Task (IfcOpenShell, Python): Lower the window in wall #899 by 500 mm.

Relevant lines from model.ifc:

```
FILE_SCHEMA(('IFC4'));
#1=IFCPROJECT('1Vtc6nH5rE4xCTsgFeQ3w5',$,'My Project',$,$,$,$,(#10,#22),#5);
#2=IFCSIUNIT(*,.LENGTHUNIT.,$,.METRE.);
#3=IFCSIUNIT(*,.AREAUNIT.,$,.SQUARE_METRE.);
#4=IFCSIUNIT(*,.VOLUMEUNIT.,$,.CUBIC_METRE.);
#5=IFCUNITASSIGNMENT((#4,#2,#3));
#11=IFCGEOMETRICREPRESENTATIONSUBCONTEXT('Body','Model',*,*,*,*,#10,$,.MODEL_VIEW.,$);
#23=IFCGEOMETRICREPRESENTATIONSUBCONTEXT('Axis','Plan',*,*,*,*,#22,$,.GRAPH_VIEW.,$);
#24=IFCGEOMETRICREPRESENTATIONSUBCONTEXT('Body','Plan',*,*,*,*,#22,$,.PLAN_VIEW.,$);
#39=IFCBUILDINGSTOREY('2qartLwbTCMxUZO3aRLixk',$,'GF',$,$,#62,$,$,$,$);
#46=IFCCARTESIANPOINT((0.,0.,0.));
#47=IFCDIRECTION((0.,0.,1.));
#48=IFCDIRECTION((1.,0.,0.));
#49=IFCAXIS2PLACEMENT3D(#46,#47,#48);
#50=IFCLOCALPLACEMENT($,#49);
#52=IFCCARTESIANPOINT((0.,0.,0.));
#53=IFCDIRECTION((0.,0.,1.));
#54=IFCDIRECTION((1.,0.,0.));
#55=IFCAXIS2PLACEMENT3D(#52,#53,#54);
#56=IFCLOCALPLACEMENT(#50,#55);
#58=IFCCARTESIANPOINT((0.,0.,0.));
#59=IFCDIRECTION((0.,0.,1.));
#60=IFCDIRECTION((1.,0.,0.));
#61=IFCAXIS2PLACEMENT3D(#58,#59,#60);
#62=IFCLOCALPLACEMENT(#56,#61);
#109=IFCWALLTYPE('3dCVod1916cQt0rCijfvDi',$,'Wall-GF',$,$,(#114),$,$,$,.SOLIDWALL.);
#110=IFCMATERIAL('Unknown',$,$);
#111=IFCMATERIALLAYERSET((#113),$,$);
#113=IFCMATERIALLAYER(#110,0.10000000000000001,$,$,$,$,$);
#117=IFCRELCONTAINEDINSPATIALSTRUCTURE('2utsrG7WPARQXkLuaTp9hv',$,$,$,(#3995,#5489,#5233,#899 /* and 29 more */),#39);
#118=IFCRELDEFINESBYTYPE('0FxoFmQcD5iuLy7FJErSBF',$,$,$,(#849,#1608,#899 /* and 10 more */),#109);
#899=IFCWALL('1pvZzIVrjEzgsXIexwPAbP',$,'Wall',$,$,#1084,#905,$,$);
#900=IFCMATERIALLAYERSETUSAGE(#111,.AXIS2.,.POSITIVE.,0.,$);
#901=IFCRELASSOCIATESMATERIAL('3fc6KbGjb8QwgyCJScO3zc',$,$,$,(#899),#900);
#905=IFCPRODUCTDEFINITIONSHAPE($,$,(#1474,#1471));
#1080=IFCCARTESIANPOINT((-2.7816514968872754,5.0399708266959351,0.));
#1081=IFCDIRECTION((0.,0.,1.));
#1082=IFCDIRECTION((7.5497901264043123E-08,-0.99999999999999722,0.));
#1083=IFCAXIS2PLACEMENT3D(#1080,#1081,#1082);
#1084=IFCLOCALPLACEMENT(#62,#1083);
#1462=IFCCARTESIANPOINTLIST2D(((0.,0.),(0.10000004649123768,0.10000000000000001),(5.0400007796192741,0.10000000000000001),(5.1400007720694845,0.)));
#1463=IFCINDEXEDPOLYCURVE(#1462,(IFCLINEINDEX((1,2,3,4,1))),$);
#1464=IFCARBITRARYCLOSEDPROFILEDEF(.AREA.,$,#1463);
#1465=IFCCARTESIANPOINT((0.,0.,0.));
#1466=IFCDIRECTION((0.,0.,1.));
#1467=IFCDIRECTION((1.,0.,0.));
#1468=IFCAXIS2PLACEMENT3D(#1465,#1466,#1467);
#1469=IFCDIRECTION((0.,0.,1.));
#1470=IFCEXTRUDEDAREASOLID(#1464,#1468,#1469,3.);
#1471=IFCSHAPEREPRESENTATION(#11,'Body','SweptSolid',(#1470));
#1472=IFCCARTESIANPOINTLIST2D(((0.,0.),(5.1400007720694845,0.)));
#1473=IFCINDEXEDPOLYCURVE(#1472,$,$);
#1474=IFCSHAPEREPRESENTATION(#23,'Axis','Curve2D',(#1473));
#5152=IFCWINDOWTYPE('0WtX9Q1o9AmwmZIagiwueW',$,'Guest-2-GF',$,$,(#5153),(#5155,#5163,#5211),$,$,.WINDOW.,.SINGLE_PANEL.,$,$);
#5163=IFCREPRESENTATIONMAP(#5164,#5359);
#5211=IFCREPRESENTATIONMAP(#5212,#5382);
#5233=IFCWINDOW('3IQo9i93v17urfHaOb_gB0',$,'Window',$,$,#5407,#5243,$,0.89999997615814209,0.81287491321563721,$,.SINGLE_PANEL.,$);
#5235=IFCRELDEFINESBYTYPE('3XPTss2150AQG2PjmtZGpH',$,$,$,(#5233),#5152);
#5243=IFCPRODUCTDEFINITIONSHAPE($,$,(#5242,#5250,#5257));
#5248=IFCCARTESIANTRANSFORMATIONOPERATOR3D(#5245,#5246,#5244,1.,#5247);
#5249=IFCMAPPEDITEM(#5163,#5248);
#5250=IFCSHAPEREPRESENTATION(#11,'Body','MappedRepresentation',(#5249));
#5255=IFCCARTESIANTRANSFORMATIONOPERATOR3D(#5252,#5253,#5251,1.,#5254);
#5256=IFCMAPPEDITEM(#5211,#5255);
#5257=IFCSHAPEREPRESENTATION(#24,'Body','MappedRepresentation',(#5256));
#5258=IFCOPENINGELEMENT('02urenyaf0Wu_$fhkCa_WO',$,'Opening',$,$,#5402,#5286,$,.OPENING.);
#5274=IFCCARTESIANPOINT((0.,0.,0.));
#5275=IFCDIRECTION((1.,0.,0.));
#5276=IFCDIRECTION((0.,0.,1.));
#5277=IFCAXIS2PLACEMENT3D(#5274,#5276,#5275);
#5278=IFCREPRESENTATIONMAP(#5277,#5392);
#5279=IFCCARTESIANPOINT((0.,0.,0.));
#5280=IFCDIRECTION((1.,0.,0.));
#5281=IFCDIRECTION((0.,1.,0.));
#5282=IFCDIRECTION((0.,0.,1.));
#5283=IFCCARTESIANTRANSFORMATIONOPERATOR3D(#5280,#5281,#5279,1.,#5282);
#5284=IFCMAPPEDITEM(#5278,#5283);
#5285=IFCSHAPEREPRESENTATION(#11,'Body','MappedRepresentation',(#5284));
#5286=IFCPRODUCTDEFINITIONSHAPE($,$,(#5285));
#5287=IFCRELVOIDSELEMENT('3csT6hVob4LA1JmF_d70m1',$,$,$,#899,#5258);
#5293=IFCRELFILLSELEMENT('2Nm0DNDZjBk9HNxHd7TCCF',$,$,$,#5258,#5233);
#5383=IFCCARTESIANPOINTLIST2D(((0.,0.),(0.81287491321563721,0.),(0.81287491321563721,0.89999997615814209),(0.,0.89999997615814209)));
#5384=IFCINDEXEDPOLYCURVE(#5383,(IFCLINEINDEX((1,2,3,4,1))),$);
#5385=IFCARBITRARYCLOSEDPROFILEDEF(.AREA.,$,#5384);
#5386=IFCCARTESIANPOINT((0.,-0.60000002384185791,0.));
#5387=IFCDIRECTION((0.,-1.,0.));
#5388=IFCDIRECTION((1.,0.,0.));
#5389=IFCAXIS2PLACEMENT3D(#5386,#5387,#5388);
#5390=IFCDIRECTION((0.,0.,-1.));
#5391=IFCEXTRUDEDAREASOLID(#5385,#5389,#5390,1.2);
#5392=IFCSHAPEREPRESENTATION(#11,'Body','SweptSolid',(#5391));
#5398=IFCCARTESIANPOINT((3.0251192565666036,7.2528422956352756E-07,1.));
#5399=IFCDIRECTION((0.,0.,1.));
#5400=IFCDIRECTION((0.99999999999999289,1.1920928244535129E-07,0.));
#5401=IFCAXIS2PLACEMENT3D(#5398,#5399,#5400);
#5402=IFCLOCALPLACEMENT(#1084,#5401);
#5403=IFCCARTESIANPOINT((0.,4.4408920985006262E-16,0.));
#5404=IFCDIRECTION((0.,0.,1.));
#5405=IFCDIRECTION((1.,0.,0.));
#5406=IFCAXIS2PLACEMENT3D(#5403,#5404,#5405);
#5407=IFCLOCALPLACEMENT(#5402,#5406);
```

```python
import numpy as np
import ifcopenshell
import ifcopenshell.api.geometry
import ifcopenshell.util.placement
import ifcopenshell.util.unit

model = ifcopenshell.open("model.ifc")
unit_scale = ifcopenshell.util.unit.calculate_unit_scale(model)

window = model.by_guid("3IQo9i93v17urfHaOb_gB0")
opening = window.FillsVoids[0].RelatingOpeningElement
dz = -0.5 / unit_scale

shift = np.array([0.0, 0.0, dz])
# The window is placed relative to its opening, so it follows when the opening moves.
matrix = ifcopenshell.util.placement.get_local_placement(opening.ObjectPlacement)
matrix[:3, 3] += shift
ifcopenshell.api.geometry.edit_object_placement(
    model, product=opening, matrix=matrix, is_si=False, should_transform_children=True
)

print(f"moved by {dz * unit_scale:+.3f} m")

model.write("model_rev.ifc")
```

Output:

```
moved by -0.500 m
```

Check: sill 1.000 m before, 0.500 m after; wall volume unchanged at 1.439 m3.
